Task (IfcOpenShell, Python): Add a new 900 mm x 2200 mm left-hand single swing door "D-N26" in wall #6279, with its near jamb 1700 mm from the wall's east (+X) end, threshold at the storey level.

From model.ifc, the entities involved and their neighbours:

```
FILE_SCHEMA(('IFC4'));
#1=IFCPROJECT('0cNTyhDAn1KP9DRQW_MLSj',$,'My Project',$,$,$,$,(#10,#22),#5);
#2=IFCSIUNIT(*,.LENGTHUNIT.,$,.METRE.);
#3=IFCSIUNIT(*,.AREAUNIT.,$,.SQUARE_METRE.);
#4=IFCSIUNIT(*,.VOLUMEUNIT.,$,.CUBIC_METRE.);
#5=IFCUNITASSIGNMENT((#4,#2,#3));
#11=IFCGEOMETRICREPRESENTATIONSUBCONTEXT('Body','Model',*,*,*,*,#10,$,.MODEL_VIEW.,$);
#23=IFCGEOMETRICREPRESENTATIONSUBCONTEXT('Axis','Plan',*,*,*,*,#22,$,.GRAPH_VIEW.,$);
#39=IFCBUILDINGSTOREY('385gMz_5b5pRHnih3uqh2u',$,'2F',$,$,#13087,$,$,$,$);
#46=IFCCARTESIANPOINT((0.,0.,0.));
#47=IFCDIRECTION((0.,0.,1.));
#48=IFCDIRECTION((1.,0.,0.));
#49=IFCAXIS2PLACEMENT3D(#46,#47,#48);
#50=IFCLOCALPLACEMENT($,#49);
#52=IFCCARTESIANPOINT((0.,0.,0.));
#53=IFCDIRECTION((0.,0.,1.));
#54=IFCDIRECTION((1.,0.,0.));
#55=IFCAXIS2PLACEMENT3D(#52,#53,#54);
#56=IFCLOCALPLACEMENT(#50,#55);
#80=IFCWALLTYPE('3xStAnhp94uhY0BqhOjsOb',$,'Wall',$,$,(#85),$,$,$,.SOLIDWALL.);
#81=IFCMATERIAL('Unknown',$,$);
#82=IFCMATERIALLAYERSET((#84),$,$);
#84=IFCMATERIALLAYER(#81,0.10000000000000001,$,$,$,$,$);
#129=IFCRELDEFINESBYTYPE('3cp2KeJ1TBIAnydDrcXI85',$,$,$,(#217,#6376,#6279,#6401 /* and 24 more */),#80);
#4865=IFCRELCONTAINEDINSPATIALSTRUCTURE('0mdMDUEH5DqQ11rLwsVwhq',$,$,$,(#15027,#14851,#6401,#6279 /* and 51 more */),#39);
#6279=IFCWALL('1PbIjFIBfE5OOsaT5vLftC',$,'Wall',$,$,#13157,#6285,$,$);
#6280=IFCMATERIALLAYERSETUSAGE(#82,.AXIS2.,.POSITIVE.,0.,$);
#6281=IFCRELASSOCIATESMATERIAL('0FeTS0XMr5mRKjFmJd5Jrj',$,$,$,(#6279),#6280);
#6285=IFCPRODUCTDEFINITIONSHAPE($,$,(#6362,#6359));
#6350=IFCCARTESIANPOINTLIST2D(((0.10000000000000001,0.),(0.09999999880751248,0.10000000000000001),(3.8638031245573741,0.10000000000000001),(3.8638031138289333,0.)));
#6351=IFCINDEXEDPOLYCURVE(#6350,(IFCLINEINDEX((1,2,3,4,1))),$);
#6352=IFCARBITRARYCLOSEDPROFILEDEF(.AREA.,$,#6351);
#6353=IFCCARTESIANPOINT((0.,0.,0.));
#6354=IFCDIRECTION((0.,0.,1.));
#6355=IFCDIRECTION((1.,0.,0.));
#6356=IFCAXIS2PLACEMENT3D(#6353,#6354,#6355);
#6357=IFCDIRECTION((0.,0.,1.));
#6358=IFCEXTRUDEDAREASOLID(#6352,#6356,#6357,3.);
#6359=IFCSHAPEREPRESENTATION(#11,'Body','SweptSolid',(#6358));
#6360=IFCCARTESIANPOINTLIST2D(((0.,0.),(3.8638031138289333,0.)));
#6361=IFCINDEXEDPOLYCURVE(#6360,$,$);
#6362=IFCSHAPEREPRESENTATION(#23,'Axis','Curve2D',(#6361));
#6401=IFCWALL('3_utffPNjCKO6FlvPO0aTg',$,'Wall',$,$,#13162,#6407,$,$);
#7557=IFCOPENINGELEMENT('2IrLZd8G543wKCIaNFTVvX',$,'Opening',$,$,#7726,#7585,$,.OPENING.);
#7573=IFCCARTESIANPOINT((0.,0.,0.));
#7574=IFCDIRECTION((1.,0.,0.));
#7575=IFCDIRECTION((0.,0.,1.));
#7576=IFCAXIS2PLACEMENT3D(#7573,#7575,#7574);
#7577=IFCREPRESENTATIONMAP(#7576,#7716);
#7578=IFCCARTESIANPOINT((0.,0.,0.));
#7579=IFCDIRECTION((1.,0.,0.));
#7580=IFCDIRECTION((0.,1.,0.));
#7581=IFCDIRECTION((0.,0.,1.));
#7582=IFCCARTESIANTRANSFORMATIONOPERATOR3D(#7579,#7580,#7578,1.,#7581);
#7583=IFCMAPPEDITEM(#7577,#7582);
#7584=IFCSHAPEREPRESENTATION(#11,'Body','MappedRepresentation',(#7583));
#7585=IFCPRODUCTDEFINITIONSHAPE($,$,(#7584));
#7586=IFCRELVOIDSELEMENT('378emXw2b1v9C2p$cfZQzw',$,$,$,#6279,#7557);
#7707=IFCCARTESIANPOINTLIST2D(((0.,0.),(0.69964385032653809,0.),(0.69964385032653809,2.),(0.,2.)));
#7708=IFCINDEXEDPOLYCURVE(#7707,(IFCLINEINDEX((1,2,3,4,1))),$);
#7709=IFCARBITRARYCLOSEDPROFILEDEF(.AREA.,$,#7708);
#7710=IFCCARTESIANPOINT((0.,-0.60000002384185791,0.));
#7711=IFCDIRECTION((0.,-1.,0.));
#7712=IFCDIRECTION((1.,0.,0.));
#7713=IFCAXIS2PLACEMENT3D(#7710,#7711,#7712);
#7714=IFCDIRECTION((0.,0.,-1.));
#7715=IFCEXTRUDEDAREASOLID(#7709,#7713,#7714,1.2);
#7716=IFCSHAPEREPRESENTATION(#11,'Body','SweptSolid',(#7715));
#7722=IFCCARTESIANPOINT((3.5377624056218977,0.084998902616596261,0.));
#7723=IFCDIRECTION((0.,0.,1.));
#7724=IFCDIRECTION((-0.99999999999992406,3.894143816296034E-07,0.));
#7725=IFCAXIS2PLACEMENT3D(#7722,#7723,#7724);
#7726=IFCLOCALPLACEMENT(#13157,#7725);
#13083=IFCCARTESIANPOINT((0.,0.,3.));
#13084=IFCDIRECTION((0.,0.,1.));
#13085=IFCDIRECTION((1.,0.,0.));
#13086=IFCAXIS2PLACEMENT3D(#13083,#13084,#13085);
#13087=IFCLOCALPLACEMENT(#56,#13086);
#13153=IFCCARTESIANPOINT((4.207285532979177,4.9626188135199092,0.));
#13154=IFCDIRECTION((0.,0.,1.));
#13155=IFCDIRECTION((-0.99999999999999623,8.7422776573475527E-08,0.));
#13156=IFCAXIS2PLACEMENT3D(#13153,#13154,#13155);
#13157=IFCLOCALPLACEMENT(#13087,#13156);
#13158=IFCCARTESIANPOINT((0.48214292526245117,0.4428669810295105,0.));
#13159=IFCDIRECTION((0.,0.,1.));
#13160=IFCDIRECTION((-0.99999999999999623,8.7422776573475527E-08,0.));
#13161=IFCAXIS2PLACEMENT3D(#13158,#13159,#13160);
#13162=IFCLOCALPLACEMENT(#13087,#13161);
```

```python
import numpy as np
import ifcopenshell
import ifcopenshell.api.feature
import ifcopenshell.api.geometry
import ifcopenshell.api.root
import ifcopenshell.api.spatial
import ifcopenshell.geom
import ifcopenshell.util.element
import ifcopenshell.util.placement
import ifcopenshell.util.representation
import ifcopenshell.util.shape
import ifcopenshell.util.unit

model = ifcopenshell.open("model.ifc")
unit_scale = ifcopenshell.util.unit.calculate_unit_scale(model)
settings = ifcopenshell.geom.settings()


def volume(element):
    """Net volume in cubic metres, openings subtracted."""
    shape = ifcopenshell.geom.create_shape(settings, element)
    return ifcopenshell.util.shape.get_volume(shape.geometry)


wall = model.by_guid("1PbIjFIBfE5OOsaT5vLftC")
storey = ifcopenshell.util.element.get_container(wall, ifc_class="IfcBuildingStorey")
context = ifcopenshell.util.representation.get_context(model, "Model", "Body", "MODEL_VIEW")
before = volume(wall)

width, height, from_end, sill = 0.9, 2.2, 1.7, 0.0  # metres

# The wall runs along its own X axis, and the end named is its -X end.
wall_shape = ifcopenshell.geom.create_shape(settings, wall)
x, y, z = ifcopenshell.util.shape.get_vertices(wall_shape.geometry).T
start = x.min() + from_end
face, thickness = float(y.min()), float(y.max() - y.min())
wall_matrix = ifcopenshell.util.placement.get_local_placement(wall.ObjectPlacement)
level = ifcopenshell.util.placement.get_local_placement(storey.ObjectPlacement)[2, 3]


def in_wall(x, y):
    """Placement at x, y metres in the wall's axes, at sill height."""
    matrix = wall_matrix.copy()
    matrix[:, 3] = wall_matrix @ np.array([x / unit_scale, y / unit_scale, 0.0, 1.0])
    matrix[2, 3] = level + sill / unit_scale
    return matrix


# Opening: a box that overshoots both wall faces by 50 mm.
opening = ifcopenshell.api.root.create_entity(model, ifc_class="IfcOpeningElement", predefined_type="OPENING")
box = ifcopenshell.api.geometry.add_wall_representation(
    model, context=context, length=width, height=height, thickness=thickness + 0.1
)
ifcopenshell.api.geometry.assign_representation(model, product=opening, representation=box)
ifcopenshell.api.geometry.edit_object_placement(model, product=opening, matrix=in_wall(start, face - 0.05), is_si=False)
ifcopenshell.api.feature.add_feature(model, feature=opening, element=wall)

door = ifcopenshell.api.root.create_entity(model, ifc_class="IfcDoor", name="D-N26", predefined_type="DOOR")
door.OverallWidth, door.OverallHeight = width / unit_scale, height / unit_scale
door.OperationType = "SINGLE_SWING_LEFT"
body = ifcopenshell.api.geometry.add_door_representation(
    model,
    context=context,
    overall_width=door.OverallWidth,
    overall_height=door.OverallHeight,
    operation_type="SINGLE_SWING_LEFT",
    lining_properties={"LiningDepth": thickness / unit_scale, "ThresholdDepth": thickness / unit_scale},
)
ifcopenshell.api.geometry.assign_representation(model, product=door, representation=body)
ifcopenshell.api.spatial.assign_container(model, products=[door], relating_structure=storey)
ifcopenshell.api.feature.add_filling(model, opening=opening, element=door)

# The lining spans the wall, so the door starts at the wall face.
ifcopenshell.api.geometry.edit_object_placement(model, product=door, matrix=in_wall(start, face), is_si=False)

after = volume(wall)

print(f"wall volume {before:.3f} -> {after:.3f} m3")

model.write("model_rev.ifc")
```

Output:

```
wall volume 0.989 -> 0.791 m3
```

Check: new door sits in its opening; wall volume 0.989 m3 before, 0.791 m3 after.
